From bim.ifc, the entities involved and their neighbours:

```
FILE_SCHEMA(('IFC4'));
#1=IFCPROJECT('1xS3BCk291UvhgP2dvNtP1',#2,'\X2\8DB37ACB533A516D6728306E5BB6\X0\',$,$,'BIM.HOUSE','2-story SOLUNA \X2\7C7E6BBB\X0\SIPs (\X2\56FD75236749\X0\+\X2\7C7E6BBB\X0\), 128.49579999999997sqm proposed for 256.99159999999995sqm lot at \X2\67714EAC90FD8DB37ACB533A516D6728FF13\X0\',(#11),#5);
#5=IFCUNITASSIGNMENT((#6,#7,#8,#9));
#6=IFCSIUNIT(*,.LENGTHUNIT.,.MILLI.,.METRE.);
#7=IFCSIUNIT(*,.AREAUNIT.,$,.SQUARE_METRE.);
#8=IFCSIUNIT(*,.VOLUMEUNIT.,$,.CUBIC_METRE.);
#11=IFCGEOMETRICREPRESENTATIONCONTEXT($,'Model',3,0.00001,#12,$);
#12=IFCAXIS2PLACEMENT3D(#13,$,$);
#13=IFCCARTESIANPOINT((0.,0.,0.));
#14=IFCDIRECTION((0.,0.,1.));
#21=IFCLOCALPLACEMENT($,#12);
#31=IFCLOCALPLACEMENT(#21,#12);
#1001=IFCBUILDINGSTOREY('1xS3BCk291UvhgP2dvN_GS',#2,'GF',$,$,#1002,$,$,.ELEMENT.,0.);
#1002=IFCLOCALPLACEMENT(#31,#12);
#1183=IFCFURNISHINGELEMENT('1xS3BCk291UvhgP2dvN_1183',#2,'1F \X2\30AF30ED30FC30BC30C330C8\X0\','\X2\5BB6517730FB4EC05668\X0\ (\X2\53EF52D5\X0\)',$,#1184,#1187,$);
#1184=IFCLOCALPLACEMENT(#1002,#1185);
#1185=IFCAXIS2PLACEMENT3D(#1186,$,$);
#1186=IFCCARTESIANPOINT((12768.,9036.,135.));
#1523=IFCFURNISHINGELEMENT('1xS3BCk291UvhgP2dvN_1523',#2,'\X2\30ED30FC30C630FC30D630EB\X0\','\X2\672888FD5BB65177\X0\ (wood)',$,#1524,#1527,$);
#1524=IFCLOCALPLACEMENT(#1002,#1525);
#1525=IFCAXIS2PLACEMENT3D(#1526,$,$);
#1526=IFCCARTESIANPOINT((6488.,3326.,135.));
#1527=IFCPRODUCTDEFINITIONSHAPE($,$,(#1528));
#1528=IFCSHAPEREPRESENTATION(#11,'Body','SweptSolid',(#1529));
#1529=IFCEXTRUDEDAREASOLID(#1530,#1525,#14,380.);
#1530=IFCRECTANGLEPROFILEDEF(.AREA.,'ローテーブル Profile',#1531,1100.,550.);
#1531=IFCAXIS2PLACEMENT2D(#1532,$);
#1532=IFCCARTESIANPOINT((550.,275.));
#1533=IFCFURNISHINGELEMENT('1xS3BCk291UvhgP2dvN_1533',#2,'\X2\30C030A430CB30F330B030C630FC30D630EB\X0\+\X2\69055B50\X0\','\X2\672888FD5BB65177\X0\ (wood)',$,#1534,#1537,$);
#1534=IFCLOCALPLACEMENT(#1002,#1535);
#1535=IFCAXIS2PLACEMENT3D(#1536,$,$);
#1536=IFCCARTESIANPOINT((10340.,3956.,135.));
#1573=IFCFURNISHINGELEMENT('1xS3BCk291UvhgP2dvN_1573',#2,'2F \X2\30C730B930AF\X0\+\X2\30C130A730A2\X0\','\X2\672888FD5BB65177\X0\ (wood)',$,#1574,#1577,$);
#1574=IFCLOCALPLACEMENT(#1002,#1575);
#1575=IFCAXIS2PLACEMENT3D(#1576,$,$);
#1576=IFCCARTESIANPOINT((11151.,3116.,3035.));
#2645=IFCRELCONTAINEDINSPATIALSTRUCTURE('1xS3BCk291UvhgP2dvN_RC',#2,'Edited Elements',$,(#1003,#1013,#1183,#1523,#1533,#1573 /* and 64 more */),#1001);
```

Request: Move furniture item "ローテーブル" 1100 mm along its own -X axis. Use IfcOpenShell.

```python
import ifcopenshell
import ifcopenshell.api.geometry
import ifcopenshell.util.placement
import ifcopenshell.util.unit

model = ifcopenshell.open("bim.ifc")
unit_scale = ifcopenshell.util.unit.calculate_unit_scale(model)

item = model.by_guid("1xS3BCk291UvhgP2dvN_1523")
matrix = ifcopenshell.util.placement.get_local_placement(item.ObjectPlacement)
matrix[:3, 3] -= matrix[:3, 0] * 1.1 / unit_scale
ifcopenshell.api.geometry.edit_object_placement(model, product=item, matrix=matrix, is_si=False)

print(ifcopenshell.util.placement.get_local_placement(item.ObjectPlacement).round(3) + 0.0)

model.write("bim_edited.ifc")
```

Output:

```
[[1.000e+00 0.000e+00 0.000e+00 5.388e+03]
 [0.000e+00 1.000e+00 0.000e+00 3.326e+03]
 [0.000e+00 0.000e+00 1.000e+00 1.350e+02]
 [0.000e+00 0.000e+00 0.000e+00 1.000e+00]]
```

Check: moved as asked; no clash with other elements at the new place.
